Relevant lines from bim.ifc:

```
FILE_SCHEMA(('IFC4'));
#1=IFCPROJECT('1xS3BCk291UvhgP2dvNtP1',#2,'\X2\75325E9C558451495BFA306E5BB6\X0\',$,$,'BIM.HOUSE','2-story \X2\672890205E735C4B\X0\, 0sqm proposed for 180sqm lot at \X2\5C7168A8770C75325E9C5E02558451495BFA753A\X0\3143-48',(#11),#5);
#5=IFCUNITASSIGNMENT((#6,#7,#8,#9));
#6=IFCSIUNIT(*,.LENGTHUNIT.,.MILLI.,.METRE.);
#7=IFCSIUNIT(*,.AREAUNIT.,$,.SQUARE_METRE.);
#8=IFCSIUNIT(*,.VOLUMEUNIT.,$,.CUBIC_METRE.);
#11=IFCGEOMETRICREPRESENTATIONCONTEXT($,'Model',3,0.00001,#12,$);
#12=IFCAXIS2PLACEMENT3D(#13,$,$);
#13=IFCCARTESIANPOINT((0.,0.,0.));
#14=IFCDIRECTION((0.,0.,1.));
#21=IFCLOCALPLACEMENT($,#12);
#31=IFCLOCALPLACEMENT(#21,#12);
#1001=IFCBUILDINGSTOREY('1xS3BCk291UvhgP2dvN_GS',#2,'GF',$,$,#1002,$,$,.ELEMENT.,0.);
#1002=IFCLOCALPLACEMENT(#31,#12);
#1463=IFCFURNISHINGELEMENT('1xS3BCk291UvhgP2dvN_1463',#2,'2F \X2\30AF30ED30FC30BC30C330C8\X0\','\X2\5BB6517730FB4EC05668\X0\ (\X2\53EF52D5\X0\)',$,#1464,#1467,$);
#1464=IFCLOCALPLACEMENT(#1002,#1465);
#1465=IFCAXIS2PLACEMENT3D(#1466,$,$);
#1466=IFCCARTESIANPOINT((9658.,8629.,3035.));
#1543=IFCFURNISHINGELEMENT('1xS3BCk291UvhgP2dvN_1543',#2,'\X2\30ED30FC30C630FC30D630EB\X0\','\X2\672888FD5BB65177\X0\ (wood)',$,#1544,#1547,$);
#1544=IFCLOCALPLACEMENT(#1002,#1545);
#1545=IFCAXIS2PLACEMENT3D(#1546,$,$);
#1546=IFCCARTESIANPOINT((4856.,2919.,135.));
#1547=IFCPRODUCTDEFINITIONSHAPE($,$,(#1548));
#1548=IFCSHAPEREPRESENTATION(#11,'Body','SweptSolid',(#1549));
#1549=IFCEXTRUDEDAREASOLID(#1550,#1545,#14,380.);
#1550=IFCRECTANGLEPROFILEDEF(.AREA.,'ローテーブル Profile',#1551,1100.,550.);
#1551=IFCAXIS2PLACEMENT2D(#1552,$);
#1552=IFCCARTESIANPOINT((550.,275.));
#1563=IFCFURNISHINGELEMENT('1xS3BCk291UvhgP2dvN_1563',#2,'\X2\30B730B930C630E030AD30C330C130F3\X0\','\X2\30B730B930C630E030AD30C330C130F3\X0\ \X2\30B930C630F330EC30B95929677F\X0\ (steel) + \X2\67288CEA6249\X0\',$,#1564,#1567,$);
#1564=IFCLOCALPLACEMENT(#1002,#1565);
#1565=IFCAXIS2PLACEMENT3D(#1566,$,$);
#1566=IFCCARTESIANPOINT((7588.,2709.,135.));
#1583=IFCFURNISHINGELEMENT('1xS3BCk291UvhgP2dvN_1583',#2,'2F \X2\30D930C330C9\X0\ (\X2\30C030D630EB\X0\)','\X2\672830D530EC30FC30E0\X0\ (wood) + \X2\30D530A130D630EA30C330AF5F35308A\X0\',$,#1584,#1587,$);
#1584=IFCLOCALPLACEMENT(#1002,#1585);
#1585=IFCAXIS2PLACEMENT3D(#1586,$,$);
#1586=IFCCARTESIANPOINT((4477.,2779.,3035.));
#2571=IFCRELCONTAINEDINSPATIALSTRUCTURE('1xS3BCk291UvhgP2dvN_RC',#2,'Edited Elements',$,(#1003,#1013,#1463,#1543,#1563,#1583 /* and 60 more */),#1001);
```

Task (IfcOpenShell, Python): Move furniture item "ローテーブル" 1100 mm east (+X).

```python
import ifcopenshell
import ifcopenshell.api.geometry
import ifcopenshell.util.placement

model = ifcopenshell.open("bim.ifc")

item = model.by_guid("1xS3BCk291UvhgP2dvN_1543")
matrix = ifcopenshell.util.placement.get_local_placement(item.ObjectPlacement)
matrix[0, 3] += 1100.0
ifcopenshell.api.geometry.edit_object_placement(model, product=item, matrix=matrix, is_si=False)

print(ifcopenshell.util.placement.get_local_placement(item.ObjectPlacement).round(3) + 0.0)

model.write("bim_rev.ifc")
```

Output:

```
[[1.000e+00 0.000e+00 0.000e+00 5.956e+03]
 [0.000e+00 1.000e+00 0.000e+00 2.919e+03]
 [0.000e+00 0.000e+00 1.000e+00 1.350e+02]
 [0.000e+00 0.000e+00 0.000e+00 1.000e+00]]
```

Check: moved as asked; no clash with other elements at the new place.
